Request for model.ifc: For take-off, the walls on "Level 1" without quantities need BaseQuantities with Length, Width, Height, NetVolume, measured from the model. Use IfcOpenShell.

First a look at what the model holds.

```python
import ifcopenshell
import ifcopenshell.util.element
import ifcopenshell.util.unit

model = ifcopenshell.open("model.ifc")
print(model.schema)
for unit_type in ("LENGTHUNIT", "AREAUNIT", "VOLUMEUNIT"):
    print(unit_type, ifcopenshell.util.unit.calculate_unit_scale(model, unit_type))
storey = next(s for s in model.by_type("IfcBuildingStorey") if s.Name == "Level 1")
walls = [e for e in ifcopenshell.util.element.get_decomposition(storey) if e.is_a("IfcWall")]
for e in sorted(walls, key=lambda e: e.id()):
    print(e.id(), e.is_a(), e.Name, list(ifcopenshell.util.element.get_psets(e, qtos_only=True)), sep=" | ")
```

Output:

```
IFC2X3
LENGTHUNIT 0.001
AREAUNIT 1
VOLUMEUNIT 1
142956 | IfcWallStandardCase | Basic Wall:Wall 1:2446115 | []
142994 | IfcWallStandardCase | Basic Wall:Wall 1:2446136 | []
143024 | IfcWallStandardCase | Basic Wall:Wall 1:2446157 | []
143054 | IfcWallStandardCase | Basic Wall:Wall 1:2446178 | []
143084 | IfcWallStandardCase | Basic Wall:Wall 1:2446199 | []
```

```python
import ifcopenshell
import ifcopenshell.api.pset
import ifcopenshell.geom
import ifcopenshell.util.element
import ifcopenshell.util.shape
import ifcopenshell.util.unit

model = ifcopenshell.open("model.ifc")
unit_scale = ifcopenshell.util.unit.calculate_unit_scale(model)
volume_scale = ifcopenshell.util.unit.calculate_unit_scale(model, "VOLUMEUNIT")
settings = ifcopenshell.geom.settings()

storey = next(s for s in model.by_type("IfcBuildingStorey") if s.Name == "Level 1")
walls = [e for e in ifcopenshell.util.element.get_decomposition(storey) if e.is_a("IfcWall")]

for e in sorted(walls, key=lambda e: e.id()):
    if ifcopenshell.util.element.get_psets(e, qtos_only=True, should_inherit=False):
        continue
    # Geometry comes back in metres, in the element's own axes.
    shape = ifcopenshell.geom.create_shape(settings, e)
    values = {
        "Length": ifcopenshell.util.shape.get_x(shape.geometry) / unit_scale,
        "Width": ifcopenshell.util.shape.get_y(shape.geometry) / unit_scale,
        "Height": ifcopenshell.util.shape.get_z(shape.geometry) / unit_scale,
        "NetVolume": ifcopenshell.util.shape.get_volume(shape.geometry) / volume_scale,
    }
    qto = ifcopenshell.api.pset.add_qto(model, product=e, name="BaseQuantities")
    ifcopenshell.api.pset.edit_qto(model, qto=qto, properties=values)
    print(e.id(), {k: round(v, 3) for k, v in values.items()})

model.write("model_edited.ifc")
```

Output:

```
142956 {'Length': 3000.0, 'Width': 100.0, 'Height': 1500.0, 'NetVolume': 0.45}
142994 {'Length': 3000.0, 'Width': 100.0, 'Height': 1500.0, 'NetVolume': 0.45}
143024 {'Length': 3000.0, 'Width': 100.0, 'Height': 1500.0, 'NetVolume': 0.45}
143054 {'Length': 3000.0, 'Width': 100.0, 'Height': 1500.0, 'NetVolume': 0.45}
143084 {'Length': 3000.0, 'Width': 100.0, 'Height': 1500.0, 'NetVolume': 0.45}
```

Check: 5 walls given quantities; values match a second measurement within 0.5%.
